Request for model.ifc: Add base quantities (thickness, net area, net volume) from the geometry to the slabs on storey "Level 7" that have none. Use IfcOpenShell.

First a look at what the model holds.

```python
import ifcopenshell
import ifcopenshell.util.element
import ifcopenshell.util.unit

model = ifcopenshell.open("model.ifc")
print(model.schema)
for unit_type in ("LENGTHUNIT", "AREAUNIT", "VOLUMEUNIT"):
    print(unit_type, ifcopenshell.util.unit.calculate_unit_scale(model, unit_type))
storey = next(s for s in model.by_type("IfcBuildingStorey") if s.Name == "Level 7")
slabs = [e for e in ifcopenshell.util.element.get_decomposition(storey) if e.is_a("IfcSlab")]
for e in sorted(slabs, key=lambda e: e.id()):
    print(e.id(), e.is_a(), e.Name, list(ifcopenshell.util.element.get_psets(e, qtos_only=True)), sep=" | ")
```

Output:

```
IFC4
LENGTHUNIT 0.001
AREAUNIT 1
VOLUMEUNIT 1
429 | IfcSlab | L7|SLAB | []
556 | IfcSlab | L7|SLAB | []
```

```python
import ifcopenshell
import ifcopenshell.api.pset
import ifcopenshell.geom
import ifcopenshell.util.element
import ifcopenshell.util.shape
import ifcopenshell.util.unit

model = ifcopenshell.open("model.ifc")
unit_scale = ifcopenshell.util.unit.calculate_unit_scale(model)
area_scale = ifcopenshell.util.unit.calculate_unit_scale(model, "AREAUNIT")
volume_scale = ifcopenshell.util.unit.calculate_unit_scale(model, "VOLUMEUNIT")
settings = ifcopenshell.geom.settings()

storey = next(s for s in model.by_type("IfcBuildingStorey") if s.Name == "Level 7")
slabs = [e for e in ifcopenshell.util.element.get_decomposition(storey) if e.is_a("IfcSlab")]

for e in sorted(slabs, key=lambda e: e.id()):
    if ifcopenshell.util.element.get_psets(e, qtos_only=True, should_inherit=False):
        continue
    # Geometry comes back in metres, in the element's own axes.
    shape = ifcopenshell.geom.create_shape(settings, e)
    values = {
        "Width": ifcopenshell.util.shape.get_z(shape.geometry) / unit_scale,
        "NetArea": ifcopenshell.util.shape.get_footprint_area(shape.geometry) / area_scale,
        "NetVolume": ifcopenshell.util.shape.get_volume(shape.geometry) / volume_scale,
    }
    qto = ifcopenshell.api.pset.add_qto(model, product=e, name="Qto_SlabBaseQuantities")
    ifcopenshell.api.pset.edit_qto(model, qto=qto, properties=values)
    print(e.id(), {k: round(v, 3) for k, v in values.items()})

model.write("model_rev.ifc")
```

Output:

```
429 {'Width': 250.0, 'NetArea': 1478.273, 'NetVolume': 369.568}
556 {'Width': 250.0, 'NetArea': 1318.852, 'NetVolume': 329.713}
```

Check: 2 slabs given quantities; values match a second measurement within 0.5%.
